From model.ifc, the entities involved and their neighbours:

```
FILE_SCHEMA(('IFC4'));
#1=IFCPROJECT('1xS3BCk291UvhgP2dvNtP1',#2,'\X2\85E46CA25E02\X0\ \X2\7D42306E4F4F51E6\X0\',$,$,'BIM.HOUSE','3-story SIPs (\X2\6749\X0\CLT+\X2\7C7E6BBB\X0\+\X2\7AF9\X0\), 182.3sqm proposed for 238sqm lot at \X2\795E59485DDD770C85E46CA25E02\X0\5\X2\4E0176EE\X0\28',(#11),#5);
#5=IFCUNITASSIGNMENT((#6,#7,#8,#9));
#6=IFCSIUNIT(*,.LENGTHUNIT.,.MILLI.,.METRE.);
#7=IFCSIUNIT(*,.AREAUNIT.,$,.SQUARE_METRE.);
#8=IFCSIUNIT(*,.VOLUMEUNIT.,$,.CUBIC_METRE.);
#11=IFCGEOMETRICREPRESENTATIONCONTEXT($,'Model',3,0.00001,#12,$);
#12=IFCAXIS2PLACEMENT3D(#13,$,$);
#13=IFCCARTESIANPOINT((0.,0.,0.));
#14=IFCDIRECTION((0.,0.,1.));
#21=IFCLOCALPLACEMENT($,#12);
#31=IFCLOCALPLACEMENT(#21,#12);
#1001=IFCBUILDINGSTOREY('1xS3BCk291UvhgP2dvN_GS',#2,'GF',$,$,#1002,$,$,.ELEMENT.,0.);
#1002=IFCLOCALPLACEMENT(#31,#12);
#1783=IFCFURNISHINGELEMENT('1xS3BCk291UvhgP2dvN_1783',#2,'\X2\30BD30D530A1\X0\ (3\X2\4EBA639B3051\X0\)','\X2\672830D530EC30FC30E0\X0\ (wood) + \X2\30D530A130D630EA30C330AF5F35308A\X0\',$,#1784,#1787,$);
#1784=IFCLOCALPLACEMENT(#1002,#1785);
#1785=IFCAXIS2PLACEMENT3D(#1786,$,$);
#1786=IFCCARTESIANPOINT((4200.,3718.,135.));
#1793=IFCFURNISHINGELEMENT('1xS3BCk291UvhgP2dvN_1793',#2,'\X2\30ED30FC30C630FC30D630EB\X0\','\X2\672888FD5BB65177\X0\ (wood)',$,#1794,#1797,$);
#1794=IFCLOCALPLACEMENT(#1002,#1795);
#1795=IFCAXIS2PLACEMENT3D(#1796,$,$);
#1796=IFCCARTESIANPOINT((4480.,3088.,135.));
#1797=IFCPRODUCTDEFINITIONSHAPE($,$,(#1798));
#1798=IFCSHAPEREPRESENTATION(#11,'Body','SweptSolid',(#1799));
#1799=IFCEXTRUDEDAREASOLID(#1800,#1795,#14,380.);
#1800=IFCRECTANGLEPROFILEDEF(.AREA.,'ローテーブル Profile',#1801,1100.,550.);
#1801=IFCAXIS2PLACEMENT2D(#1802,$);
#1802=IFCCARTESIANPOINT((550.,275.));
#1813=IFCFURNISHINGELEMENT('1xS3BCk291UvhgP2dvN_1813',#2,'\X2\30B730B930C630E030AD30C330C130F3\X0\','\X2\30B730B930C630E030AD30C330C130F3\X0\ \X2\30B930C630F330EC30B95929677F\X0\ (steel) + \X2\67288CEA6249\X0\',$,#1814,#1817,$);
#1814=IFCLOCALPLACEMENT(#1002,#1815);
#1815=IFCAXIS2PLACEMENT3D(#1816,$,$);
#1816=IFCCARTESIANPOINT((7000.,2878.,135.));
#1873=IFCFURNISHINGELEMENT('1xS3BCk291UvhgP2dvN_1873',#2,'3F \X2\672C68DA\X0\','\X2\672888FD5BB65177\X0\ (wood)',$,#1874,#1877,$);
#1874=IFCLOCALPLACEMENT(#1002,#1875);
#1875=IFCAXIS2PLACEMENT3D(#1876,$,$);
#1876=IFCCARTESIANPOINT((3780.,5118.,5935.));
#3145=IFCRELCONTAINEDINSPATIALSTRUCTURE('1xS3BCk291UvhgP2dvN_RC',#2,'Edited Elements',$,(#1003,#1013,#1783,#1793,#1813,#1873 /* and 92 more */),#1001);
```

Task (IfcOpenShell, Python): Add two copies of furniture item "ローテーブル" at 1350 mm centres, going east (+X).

```python
import numpy as np
import ifcopenshell
import ifcopenshell.api.geometry
import ifcopenshell.api.root
import ifcopenshell.util.element
import ifcopenshell.util.placement

model = ifcopenshell.open("model.ifc")


def reuse_history(source, copy):
    """copy_class also copies each property set's owner history, people and application; keep the originals."""
    for rel in copy.IsDefinedBy:
        if rel.is_a("IfcRelDefinesByProperties") and (history := rel.RelatingPropertyDefinition.OwnerHistory):
            rel.RelatingPropertyDefinition.OwnerHistory = source.OwnerHistory
            ifcopenshell.util.element.remove_deep2(model, history)


source = model.by_guid("1xS3BCk291UvhgP2dvN_1793")
base = ifcopenshell.util.placement.get_local_placement(source.ObjectPlacement)
step = np.array([1.0, 0.0, 0.0]) * 1350.0

for i in range(1, 3):
    copy = ifcopenshell.api.root.copy_class(model, product=source)
    copy.Representation = ifcopenshell.util.element.copy_deep(
        model, source.Representation, exclude=["IfcGeometricRepresentationContext", "IfcRepresentationMap"]
    )
    reuse_history(source, copy)
    matrix = base.copy()
    matrix[:3, 3] += i * step
    print("added at", matrix[:3, 3].round(3) + 0.0)
    ifcopenshell.api.geometry.edit_object_placement(model, product=copy, matrix=matrix, is_si=False)

model.write("model_rev.ifc")
```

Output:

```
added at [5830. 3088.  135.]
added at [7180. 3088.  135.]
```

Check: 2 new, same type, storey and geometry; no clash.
